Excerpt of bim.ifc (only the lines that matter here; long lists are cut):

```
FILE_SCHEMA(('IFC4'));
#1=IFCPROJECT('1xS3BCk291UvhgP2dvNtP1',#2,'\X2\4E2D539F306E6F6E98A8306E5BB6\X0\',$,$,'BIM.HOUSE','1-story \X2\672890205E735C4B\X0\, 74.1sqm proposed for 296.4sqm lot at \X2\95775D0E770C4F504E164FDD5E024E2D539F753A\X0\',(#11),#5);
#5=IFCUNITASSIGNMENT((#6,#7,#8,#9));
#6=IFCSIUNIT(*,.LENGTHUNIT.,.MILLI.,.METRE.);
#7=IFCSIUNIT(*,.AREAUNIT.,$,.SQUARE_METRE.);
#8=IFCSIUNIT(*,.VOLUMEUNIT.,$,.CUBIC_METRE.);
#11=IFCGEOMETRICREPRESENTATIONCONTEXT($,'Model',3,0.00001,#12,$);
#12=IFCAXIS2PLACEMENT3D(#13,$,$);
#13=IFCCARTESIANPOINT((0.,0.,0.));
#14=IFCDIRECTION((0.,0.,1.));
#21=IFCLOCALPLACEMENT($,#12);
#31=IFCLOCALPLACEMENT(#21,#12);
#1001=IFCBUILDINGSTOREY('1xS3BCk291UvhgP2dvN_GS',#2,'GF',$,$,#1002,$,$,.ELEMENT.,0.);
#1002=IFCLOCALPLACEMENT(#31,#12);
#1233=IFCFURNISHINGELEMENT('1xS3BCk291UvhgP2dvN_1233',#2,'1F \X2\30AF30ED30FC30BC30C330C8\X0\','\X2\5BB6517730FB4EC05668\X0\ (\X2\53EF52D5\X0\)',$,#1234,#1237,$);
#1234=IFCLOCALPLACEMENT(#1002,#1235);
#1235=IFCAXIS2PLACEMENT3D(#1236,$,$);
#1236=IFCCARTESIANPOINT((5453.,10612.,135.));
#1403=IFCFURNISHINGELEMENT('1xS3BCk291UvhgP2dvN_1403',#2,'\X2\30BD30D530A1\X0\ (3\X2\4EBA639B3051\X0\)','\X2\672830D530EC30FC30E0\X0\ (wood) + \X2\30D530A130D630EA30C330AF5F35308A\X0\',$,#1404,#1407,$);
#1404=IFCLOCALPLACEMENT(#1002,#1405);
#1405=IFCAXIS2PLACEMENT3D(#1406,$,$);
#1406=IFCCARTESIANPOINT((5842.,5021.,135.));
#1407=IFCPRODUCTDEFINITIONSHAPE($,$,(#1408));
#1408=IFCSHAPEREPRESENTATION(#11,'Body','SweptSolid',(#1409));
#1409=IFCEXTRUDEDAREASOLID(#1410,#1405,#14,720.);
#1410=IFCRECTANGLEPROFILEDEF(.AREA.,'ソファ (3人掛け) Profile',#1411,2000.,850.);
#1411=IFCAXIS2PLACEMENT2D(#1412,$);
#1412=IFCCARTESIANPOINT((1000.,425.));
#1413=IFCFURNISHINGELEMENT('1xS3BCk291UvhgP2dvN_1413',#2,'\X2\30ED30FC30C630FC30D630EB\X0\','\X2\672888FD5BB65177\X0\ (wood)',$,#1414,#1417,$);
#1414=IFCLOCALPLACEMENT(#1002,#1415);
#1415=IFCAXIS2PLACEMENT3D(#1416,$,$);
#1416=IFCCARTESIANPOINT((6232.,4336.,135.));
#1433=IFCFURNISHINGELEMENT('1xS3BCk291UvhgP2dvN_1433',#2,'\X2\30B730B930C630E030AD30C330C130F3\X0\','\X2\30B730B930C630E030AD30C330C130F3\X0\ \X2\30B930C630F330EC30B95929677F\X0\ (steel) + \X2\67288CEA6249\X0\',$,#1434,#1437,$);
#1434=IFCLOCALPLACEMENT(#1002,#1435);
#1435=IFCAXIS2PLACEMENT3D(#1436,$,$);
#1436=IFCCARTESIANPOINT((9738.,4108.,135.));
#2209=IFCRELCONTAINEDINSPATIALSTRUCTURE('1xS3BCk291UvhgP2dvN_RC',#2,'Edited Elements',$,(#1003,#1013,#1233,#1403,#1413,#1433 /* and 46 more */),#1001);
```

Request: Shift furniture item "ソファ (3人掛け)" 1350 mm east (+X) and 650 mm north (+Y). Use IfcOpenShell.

```python
import ifcopenshell
import ifcopenshell.api.geometry
import ifcopenshell.util.placement
import ifcopenshell.util.unit

model = ifcopenshell.open("bim.ifc")
unit_scale = ifcopenshell.util.unit.calculate_unit_scale(model)

item = model.by_guid("1xS3BCk291UvhgP2dvN_1403")
matrix = ifcopenshell.util.placement.get_local_placement(item.ObjectPlacement)
matrix[0, 3] += 1.35 / unit_scale
matrix[1, 3] += 0.65 / unit_scale
ifcopenshell.api.geometry.edit_object_placement(model, product=item, matrix=matrix, is_si=False)

print(ifcopenshell.util.placement.get_local_placement(item.ObjectPlacement).round(3) + 0.0)

model.write("bim-out.ifc")
```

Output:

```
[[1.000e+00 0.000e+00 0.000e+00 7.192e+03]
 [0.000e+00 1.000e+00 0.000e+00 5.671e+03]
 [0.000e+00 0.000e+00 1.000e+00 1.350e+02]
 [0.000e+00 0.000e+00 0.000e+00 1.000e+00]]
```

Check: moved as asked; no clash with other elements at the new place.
